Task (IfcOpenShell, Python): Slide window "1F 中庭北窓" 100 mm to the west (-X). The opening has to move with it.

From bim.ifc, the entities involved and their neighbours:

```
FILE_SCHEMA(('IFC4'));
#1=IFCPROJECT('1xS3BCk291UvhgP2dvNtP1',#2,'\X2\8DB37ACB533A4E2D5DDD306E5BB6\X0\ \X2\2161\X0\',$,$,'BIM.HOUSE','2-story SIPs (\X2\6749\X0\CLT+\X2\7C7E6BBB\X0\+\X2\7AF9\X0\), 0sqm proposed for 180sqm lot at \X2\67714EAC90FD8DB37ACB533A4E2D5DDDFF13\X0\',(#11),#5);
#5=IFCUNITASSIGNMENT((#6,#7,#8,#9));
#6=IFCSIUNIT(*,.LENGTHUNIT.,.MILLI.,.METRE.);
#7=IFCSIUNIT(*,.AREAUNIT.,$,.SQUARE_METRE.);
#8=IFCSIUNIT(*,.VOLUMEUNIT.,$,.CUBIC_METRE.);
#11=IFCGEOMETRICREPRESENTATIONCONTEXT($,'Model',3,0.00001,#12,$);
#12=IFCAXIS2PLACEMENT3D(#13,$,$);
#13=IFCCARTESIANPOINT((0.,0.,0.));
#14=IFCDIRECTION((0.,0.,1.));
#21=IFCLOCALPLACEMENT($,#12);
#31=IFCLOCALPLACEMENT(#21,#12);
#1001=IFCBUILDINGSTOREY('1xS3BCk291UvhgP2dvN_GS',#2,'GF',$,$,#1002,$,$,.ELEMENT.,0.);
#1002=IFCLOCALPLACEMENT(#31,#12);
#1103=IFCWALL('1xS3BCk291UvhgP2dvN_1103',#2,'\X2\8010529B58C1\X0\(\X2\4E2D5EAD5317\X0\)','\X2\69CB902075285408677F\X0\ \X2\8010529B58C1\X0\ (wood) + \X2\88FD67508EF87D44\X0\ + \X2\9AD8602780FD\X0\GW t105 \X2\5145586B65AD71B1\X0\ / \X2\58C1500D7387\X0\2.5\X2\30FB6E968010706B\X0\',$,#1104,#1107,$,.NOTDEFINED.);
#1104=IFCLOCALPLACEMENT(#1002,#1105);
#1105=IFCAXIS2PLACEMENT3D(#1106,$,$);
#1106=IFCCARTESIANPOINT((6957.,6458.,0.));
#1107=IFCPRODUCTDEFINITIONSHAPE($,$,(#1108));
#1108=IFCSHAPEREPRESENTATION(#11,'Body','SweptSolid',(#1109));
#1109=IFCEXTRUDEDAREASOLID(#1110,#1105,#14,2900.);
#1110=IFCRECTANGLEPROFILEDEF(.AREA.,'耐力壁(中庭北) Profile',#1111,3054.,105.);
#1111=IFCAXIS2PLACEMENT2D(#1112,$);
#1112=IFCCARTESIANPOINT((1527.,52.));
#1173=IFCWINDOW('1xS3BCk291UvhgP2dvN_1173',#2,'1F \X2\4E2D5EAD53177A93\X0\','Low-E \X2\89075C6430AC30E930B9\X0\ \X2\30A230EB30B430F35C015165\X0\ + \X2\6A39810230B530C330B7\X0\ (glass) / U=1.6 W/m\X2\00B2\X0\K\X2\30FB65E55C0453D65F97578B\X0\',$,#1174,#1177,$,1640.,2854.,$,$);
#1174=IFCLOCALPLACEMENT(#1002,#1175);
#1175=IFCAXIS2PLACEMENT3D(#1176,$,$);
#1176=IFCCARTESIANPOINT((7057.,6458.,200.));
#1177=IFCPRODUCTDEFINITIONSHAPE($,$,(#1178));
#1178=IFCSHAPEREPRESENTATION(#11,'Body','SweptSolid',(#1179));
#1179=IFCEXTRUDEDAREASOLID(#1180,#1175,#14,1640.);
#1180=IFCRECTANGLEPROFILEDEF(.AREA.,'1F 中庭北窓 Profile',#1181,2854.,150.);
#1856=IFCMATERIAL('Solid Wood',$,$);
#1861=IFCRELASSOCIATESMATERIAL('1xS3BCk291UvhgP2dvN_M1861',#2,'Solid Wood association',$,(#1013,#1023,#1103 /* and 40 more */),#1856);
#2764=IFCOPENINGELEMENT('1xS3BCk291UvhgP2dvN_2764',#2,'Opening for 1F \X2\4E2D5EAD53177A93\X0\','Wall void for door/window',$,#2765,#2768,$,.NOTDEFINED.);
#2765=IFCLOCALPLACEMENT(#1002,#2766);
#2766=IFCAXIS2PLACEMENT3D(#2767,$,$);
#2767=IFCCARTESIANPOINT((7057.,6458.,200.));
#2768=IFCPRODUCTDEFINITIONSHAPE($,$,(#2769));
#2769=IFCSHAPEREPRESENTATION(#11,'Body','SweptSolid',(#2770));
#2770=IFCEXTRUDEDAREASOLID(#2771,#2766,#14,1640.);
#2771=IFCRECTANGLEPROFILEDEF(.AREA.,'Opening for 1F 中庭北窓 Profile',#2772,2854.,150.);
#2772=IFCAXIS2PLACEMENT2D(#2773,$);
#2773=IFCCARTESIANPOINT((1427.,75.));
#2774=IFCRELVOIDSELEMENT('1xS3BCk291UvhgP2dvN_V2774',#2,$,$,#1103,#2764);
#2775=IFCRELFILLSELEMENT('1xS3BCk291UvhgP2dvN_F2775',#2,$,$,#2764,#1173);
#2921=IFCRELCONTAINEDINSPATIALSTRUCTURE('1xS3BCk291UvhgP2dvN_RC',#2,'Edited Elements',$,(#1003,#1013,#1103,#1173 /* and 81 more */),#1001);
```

```python
import ifcopenshell
import ifcopenshell.api.geometry
import ifcopenshell.util.placement

model = ifcopenshell.open("bim.ifc")

window = model.by_guid("1xS3BCk291UvhgP2dvN_1173")
opening = window.FillsVoids[0].RelatingOpeningElement
wall = opening.VoidsElements[0].RelatingBuildingElement

wall_matrix = ifcopenshell.util.placement.get_local_placement(wall.ObjectPlacement)
shift = wall_matrix[:3, 0] * -100.0
before = ifcopenshell.util.placement.get_local_placement(window.ObjectPlacement)[:3, 3].copy()

# The window is not placed relative to its opening, so move both.
for product in (opening, window):
    matrix = ifcopenshell.util.placement.get_local_placement(product.ObjectPlacement)
    matrix[:3, 3] += shift
    ifcopenshell.api.geometry.edit_object_placement(model, product=product, matrix=matrix, is_si=False)

after = ifcopenshell.util.placement.get_local_placement(window.ObjectPlacement)[:3, 3]
print("window moved by", (after - before).round(3) + 0.0)

model.write("bim-out.ifc")
```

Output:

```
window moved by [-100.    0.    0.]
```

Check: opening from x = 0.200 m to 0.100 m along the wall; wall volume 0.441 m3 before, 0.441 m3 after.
